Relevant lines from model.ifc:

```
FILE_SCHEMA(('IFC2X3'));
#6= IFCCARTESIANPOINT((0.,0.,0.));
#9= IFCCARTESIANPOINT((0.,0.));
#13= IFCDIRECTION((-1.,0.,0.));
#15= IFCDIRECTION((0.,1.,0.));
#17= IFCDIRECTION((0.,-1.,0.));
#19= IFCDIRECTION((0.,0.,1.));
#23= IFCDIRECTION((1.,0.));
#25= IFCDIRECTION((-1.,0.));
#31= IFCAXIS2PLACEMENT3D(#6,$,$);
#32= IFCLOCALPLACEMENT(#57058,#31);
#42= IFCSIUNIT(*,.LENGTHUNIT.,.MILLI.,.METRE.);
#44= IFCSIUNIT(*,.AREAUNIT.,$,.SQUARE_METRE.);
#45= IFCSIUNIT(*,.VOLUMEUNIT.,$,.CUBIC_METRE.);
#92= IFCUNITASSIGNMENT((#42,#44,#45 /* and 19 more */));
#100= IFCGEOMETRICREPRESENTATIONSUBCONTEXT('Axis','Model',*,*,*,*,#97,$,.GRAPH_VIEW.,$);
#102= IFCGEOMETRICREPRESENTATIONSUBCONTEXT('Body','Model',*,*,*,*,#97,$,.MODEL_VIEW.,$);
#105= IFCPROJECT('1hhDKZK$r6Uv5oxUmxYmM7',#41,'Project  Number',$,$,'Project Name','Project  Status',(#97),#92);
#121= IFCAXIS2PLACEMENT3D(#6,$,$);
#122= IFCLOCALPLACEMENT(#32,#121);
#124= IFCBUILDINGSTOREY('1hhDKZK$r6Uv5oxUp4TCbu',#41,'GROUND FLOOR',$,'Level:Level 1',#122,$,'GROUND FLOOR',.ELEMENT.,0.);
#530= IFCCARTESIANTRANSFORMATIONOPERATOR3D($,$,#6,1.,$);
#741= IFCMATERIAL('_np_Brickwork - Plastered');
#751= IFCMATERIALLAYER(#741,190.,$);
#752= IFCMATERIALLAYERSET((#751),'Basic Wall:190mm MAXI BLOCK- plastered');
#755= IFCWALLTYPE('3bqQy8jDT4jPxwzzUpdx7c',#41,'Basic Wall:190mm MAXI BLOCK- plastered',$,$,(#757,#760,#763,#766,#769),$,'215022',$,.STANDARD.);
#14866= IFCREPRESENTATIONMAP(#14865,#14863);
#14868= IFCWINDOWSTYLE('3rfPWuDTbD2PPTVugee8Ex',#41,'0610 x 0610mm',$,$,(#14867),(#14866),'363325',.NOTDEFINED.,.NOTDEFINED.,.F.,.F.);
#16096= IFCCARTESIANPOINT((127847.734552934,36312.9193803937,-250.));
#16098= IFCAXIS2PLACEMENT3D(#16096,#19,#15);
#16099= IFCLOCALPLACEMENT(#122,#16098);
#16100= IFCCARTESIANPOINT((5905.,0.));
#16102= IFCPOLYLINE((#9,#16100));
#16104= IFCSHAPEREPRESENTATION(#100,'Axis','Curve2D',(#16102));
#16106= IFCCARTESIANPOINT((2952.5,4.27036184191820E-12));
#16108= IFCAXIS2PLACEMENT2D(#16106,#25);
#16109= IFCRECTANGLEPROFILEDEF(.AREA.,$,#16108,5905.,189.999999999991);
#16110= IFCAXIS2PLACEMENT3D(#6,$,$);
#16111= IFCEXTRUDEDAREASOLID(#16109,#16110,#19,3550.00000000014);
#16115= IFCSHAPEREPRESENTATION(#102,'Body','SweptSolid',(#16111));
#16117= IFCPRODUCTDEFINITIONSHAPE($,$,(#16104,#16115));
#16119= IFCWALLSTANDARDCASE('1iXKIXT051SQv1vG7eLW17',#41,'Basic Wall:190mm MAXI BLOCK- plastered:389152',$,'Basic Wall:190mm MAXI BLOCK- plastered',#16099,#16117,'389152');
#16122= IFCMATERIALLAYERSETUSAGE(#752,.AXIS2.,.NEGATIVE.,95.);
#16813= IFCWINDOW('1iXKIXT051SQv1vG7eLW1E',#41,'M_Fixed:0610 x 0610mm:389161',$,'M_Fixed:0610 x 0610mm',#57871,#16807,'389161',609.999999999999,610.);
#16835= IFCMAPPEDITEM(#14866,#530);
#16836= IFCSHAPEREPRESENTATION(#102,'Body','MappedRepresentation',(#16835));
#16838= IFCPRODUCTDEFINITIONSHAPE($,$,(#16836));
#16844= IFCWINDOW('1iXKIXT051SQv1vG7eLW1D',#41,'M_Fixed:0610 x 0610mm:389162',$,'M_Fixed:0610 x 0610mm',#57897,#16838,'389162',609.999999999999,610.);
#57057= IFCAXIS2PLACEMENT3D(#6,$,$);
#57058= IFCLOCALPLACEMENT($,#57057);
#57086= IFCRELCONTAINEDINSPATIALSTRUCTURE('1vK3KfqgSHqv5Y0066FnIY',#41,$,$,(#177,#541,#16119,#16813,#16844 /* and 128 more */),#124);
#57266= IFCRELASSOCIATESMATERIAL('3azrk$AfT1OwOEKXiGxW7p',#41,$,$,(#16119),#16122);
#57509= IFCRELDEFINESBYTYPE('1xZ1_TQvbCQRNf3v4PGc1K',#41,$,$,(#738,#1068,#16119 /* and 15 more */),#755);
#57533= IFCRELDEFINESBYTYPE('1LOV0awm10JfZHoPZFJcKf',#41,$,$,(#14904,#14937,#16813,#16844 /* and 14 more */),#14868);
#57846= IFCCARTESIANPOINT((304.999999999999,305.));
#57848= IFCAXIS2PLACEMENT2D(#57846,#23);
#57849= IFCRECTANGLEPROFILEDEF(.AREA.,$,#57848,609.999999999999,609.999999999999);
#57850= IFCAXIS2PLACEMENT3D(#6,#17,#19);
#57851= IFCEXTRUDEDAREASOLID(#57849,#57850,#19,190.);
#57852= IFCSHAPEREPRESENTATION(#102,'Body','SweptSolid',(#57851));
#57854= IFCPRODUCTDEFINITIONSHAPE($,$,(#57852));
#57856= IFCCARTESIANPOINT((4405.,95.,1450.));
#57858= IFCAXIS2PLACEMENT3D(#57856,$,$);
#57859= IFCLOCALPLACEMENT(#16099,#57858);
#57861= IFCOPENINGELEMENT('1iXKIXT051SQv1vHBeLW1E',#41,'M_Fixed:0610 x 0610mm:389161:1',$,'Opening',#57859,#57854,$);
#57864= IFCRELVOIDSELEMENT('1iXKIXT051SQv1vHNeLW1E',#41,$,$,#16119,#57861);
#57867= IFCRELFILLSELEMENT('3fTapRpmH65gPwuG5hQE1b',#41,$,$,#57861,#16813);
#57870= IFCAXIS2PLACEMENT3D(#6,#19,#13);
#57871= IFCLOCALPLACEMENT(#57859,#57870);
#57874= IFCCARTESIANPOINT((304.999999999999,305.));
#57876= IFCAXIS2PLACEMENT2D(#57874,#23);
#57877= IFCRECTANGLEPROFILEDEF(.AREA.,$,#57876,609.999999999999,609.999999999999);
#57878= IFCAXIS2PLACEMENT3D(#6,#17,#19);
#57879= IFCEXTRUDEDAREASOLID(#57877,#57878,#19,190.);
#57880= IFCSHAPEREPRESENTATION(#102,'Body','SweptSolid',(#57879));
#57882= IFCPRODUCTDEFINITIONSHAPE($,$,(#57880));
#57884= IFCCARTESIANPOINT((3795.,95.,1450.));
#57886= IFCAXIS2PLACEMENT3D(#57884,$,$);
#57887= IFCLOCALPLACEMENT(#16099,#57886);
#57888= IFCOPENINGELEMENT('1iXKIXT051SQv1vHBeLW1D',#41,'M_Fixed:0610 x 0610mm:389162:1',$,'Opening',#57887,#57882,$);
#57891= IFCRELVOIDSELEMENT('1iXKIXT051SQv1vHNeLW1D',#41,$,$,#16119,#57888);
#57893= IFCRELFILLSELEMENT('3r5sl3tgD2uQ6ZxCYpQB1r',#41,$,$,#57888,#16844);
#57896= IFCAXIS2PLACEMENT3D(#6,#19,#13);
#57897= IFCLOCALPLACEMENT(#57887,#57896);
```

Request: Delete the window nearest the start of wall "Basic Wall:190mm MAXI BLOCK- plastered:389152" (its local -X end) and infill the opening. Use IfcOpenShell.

```python
import ifcopenshell
import ifcopenshell.api.feature
import ifcopenshell.api.root
import ifcopenshell.geom
import ifcopenshell.util.shape

model = ifcopenshell.open("model.ifc")
settings = ifcopenshell.geom.settings()


def volume(element):
    """Net volume in cubic metres, openings subtracted."""
    shape = ifcopenshell.geom.create_shape(settings, element)
    return ifcopenshell.util.shape.get_volume(shape.geometry)


window = model.by_guid("1iXKIXT051SQv1vG7eLW1D")
opening = window.FillsVoids[0].RelatingOpeningElement
wall = opening.VoidsElements[0].RelatingBuildingElement
before = volume(wall)

ifcopenshell.api.root.remove_product(model, product=window)
ifcopenshell.api.feature.remove_feature(model, feature=opening)

after = volume(wall)

print(f"wall volume {before:.3f} -> {after:.3f} m3")

model.write("model-out.ifc")
```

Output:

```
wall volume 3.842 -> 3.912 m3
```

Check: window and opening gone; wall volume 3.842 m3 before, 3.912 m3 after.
